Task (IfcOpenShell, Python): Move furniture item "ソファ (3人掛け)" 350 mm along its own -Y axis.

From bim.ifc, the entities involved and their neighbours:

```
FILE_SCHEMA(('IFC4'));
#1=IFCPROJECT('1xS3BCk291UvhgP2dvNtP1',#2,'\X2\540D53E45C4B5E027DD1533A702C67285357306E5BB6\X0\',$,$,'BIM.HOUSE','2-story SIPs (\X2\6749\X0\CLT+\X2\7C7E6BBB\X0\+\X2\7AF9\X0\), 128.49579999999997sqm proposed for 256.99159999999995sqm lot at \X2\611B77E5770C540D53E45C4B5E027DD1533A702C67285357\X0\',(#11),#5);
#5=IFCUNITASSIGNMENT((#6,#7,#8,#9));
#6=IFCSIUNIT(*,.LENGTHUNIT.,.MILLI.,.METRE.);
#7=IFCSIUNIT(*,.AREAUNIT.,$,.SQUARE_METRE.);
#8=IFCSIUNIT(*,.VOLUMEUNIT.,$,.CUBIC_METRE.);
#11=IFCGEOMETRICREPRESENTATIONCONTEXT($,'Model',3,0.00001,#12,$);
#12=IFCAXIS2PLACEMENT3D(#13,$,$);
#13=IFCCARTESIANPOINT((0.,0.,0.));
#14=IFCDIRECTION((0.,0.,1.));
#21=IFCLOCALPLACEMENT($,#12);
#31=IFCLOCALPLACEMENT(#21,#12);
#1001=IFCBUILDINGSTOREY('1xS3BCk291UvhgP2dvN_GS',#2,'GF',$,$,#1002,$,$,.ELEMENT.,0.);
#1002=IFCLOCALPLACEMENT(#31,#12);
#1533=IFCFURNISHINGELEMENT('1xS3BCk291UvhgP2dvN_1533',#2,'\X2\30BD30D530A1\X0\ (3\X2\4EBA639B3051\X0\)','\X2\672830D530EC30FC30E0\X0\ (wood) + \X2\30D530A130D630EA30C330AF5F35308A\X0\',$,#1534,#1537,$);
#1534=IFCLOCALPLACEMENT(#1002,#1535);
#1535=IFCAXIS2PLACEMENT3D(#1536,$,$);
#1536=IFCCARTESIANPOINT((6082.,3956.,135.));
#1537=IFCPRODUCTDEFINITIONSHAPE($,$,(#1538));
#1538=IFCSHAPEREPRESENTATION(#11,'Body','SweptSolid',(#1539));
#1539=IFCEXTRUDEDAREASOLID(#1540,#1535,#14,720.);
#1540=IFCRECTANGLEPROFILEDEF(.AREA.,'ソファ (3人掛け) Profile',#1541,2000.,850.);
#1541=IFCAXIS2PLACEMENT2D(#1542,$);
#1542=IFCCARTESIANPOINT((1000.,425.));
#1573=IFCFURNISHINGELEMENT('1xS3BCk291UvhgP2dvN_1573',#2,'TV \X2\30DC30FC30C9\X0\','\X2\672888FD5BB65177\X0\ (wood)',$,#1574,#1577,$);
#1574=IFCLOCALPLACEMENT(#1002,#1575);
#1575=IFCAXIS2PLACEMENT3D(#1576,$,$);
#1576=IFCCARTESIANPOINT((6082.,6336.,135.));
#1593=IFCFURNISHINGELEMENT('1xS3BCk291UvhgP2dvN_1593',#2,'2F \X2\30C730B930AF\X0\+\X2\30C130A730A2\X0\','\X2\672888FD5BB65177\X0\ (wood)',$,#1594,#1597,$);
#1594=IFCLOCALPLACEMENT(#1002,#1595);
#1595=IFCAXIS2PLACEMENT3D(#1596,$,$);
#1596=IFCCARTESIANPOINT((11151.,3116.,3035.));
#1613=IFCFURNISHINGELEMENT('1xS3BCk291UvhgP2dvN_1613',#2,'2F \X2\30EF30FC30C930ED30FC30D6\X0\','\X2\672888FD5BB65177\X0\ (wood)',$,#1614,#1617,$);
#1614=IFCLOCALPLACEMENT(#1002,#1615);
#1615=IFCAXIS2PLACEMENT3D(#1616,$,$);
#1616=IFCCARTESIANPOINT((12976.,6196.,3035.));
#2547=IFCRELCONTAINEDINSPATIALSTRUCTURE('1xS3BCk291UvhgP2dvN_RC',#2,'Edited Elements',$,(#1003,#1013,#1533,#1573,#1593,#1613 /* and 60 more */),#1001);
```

```python
import ifcopenshell
import ifcopenshell.api.geometry
import ifcopenshell.util.placement

model = ifcopenshell.open("bim.ifc")

item = model.by_guid("1xS3BCk291UvhgP2dvN_1533")
matrix = ifcopenshell.util.placement.get_local_placement(item.ObjectPlacement)
matrix[:3, 3] -= matrix[:3, 1] * 350.0
ifcopenshell.api.geometry.edit_object_placement(model, product=item, matrix=matrix, is_si=False)

print(ifcopenshell.util.placement.get_local_placement(item.ObjectPlacement).round(3) + 0.0)

model.write("bim_updated.ifc")
```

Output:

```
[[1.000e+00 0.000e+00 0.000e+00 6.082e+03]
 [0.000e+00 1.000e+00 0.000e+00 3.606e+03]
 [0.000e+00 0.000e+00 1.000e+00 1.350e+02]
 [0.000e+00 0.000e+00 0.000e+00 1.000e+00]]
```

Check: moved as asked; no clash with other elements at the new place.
